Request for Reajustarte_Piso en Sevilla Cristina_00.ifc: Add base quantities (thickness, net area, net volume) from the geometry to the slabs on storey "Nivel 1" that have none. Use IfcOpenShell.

First a look at what the model holds.

```python
import ifcopenshell
import ifcopenshell.util.element
import ifcopenshell.util.unit

model = ifcopenshell.open("Reajustarte_Piso en Sevilla Cristina_00.ifc")
print(model.schema)
for unit_type in ("LENGTHUNIT", "AREAUNIT", "VOLUMEUNIT"):
    print(unit_type, ifcopenshell.util.unit.calculate_unit_scale(model, unit_type))
storey = next(s for s in model.by_type("IfcBuildingStorey") if s.Name == "Nivel 1")
slabs = [e for e in ifcopenshell.util.element.get_decomposition(storey) if e.is_a("IfcSlab")]
for e in sorted(slabs, key=lambda e: e.id()):
    print(e.id(), e.is_a(), e.Name, list(ifcopenshell.util.element.get_psets(e, qtos_only=True)), sep=" | ")
```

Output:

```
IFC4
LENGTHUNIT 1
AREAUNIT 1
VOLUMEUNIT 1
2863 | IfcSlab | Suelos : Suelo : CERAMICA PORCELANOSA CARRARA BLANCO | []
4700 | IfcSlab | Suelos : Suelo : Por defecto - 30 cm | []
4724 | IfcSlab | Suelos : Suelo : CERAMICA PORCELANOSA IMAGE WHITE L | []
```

```python
import ifcopenshell
import ifcopenshell.api.pset
import ifcopenshell.geom
import ifcopenshell.util.element
import ifcopenshell.util.shape
import ifcopenshell.util.unit

model = ifcopenshell.open("Reajustarte_Piso en Sevilla Cristina_00.ifc")
unit_scale = ifcopenshell.util.unit.calculate_unit_scale(model)
area_scale = ifcopenshell.util.unit.calculate_unit_scale(model, "AREAUNIT")
volume_scale = ifcopenshell.util.unit.calculate_unit_scale(model, "VOLUMEUNIT")
settings = ifcopenshell.geom.settings()

storey = next(s for s in model.by_type("IfcBuildingStorey") if s.Name == "Nivel 1")
slabs = [e for e in ifcopenshell.util.element.get_decomposition(storey) if e.is_a("IfcSlab")]

for e in sorted(slabs, key=lambda e: e.id()):
    if ifcopenshell.util.element.get_psets(e, qtos_only=True, should_inherit=False):
        continue
    # Geometry comes back in metres, in the element's own axes.
    shape = ifcopenshell.geom.create_shape(settings, e)
    values = {
        "Width": ifcopenshell.util.shape.get_z(shape.geometry) / unit_scale,
        "NetArea": ifcopenshell.util.shape.get_footprint_area(shape.geometry) / area_scale,
        "NetVolume": ifcopenshell.util.shape.get_volume(shape.geometry) / volume_scale,
    }
    qto = ifcopenshell.api.pset.add_qto(model, product=e, name="Qto_SlabBaseQuantities")
    ifcopenshell.api.pset.edit_qto(model, qto=qto, properties=values)
    print(e.id(), {k: round(v, 3) for k, v in values.items()})

model.write("Reajustarte_Piso en Sevilla Cristina_00-out.ifc")
```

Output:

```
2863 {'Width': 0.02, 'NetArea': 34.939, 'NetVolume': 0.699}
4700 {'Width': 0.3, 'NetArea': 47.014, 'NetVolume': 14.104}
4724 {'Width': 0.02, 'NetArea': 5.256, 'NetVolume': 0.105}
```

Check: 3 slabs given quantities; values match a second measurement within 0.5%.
